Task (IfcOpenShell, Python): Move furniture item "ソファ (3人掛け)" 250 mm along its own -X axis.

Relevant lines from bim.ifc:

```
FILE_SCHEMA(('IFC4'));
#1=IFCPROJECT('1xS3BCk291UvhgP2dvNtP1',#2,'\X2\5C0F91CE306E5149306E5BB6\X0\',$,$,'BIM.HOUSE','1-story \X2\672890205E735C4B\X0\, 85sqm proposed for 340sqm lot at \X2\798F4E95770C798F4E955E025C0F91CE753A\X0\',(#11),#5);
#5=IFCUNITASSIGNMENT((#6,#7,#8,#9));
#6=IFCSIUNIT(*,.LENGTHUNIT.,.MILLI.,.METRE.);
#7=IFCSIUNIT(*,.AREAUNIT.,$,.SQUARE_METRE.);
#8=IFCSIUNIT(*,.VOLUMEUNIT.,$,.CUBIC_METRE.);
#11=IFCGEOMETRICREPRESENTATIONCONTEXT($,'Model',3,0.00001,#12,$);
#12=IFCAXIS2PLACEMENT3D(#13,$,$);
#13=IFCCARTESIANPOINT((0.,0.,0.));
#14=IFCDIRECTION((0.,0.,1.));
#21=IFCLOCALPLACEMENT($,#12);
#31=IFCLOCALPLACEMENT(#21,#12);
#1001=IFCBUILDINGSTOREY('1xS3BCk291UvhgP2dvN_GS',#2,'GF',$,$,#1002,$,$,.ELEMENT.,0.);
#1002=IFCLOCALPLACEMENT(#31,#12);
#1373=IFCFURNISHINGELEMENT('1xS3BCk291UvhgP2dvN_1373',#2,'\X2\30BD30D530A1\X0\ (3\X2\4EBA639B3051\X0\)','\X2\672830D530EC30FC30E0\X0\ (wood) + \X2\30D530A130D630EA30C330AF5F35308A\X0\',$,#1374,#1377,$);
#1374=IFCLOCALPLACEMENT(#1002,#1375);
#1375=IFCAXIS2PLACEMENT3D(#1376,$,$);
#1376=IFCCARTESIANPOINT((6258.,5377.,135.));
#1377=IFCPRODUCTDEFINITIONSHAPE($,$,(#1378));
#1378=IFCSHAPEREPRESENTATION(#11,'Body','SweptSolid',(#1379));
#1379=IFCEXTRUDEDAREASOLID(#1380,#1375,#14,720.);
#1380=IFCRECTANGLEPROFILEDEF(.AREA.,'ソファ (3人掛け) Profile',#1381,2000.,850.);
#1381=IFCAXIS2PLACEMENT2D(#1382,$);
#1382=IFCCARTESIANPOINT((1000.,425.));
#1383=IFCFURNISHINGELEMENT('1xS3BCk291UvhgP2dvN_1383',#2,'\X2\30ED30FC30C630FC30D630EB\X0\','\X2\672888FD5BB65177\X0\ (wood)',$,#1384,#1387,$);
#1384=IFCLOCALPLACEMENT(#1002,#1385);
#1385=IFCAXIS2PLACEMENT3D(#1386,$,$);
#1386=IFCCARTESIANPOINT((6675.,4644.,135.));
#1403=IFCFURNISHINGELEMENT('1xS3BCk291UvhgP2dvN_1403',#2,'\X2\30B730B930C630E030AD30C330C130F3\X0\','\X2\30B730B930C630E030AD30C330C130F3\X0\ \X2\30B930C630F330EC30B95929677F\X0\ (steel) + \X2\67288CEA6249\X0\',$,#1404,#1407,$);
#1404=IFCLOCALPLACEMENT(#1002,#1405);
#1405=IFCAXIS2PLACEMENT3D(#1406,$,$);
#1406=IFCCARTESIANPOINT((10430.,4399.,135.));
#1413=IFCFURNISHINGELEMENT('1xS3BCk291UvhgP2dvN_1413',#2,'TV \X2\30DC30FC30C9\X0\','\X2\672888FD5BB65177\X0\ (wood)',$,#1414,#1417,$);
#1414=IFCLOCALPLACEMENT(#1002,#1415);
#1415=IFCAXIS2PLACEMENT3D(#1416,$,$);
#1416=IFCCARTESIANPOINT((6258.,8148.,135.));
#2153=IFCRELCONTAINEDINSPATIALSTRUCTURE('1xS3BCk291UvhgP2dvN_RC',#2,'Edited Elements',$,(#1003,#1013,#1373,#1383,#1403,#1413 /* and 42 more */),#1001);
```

```python
import ifcopenshell
import ifcopenshell.api.geometry
import ifcopenshell.util.placement

model = ifcopenshell.open("bim.ifc")

item = model.by_id(1373)
matrix = ifcopenshell.util.placement.get_local_placement(item.ObjectPlacement)
matrix[:3, 3] -= matrix[:3, 0] * 250.0
ifcopenshell.api.geometry.edit_object_placement(model, product=item, matrix=matrix, is_si=False)

print(ifcopenshell.util.placement.get_local_placement(item.ObjectPlacement).round(3) + 0.0)

model.write("bim_updated.ifc")
```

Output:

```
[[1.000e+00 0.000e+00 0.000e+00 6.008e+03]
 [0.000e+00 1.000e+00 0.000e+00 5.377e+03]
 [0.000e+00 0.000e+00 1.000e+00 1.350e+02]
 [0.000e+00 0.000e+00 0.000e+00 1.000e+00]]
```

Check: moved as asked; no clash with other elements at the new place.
